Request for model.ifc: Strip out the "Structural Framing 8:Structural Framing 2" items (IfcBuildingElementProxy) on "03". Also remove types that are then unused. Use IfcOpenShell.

First a look at what the model holds.

```python
import ifcopenshell
import ifcopenshell.util.element

model = ifcopenshell.open("model.ifc")
print(model.schema)
storey = next(s for s in model.by_type("IfcBuildingStorey") if s.Name == "03")
proxies = [e for e in ifcopenshell.util.element.get_decomposition(storey) if e.is_a("IfcBuildingElementProxy")]
seen = {}
for e in proxies:
    element_type = ifcopenshell.util.element.get_type(e)
    name = element_type.Name if element_type not in (None, e) else None
    seen[name] = seen.get(name, 0) + 1
for name, count in sorted(seen.items(), key=str):
    print(count, "x", name)
```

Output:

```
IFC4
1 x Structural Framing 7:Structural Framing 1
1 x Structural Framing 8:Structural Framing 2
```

```python
import ifcopenshell
import ifcopenshell.api.root
import ifcopenshell.util.element

model = ifcopenshell.open("model.ifc")

storey = next(s for s in model.by_type("IfcBuildingStorey") if s.Name == "03")
proxies = [e for e in ifcopenshell.util.element.get_decomposition(storey) if e.is_a("IfcBuildingElementProxy")]
targets = [e for e in proxies if (t := ifcopenshell.util.element.get_type(e)) not in (None, e) and t.Name == "Structural Framing 8:Structural Framing 2"]
types = {ifcopenshell.util.element.get_type(e) for e in targets} - {None, *targets}

for e in targets:
    ifcopenshell.api.root.remove_product(model, product=e)
print(len(targets), "removed")

unused = [t for t in types if not ifcopenshell.util.element.get_types(t)]
for t in unused:
    ifcopenshell.api.root.remove_product(model, product=t)
print(len(unused), "unused types removed")

model.write("model_rev.ifc")
```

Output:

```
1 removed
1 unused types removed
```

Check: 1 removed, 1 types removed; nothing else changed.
